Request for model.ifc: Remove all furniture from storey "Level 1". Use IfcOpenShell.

First a look at what the model holds.

```python
import ifcopenshell
import ifcopenshell.util.element

model = ifcopenshell.open("model.ifc")
print(model.schema)
storey = next(s for s in model.by_type("IfcBuildingStorey") if s.Name == "Level 1")
furniture = [e for e in ifcopenshell.util.element.get_decomposition(storey) if e.is_a("IfcFurnishingElement")]
seen = {}
for e in furniture:
    element_type = ifcopenshell.util.element.get_type(e)
    name = element_type.Name if element_type not in (None, e) else None
    seen[name] = seen.get(name, 0) + 1
for name, count in sorted(seen.items(), key=str):
    print(count, "x", name)
```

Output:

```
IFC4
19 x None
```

```python
import ifcopenshell
import ifcopenshell.api.root
import ifcopenshell.util.element

model = ifcopenshell.open("model.ifc")

storey = next(s for s in model.by_type("IfcBuildingStorey") if s.Name == "Level 1")
furniture = [e for e in ifcopenshell.util.element.get_decomposition(storey) if e.is_a("IfcFurnishingElement")]

for e in furniture:
    ifcopenshell.api.root.remove_product(model, product=e)
print(len(furniture), "removed")

model.write("model_rev.ifc")
```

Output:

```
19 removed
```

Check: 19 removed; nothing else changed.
